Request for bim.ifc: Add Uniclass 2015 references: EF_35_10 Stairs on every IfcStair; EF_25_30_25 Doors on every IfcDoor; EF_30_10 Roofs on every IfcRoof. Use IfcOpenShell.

First a look at what the model holds.

```python
import ifcopenshell

model = ifcopenshell.open("bim.ifc")
print(model.schema)
print("classifications:", [c.Name for c in model.by_type("IfcClassification")])
for ifc_class in ("IfcDoor", "IfcRoof", "IfcStair", "IfcWall", "IfcWindow"):
    print(ifc_class, len(model.by_type(ifc_class)))
```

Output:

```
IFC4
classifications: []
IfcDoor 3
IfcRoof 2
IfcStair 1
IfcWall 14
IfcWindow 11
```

```python
import ifcopenshell
import ifcopenshell.api.classification

model = ifcopenshell.open("bim.ifc")

system = ifcopenshell.api.classification.add_classification(model, classification="Uniclass 2015")

codes = {
    "IfcStair": ("EF_35_10", "Stairs"),
    "IfcDoor": ("EF_25_30_25", "Doors"),
    "IfcRoof": ("EF_30_10", "Roofs"),
}
for ifc_class, (code, name) in codes.items():
    products = model.by_type(ifc_class)
    ifcopenshell.api.classification.add_reference(
        model, products=products, classification=system, identification=code, name=name
    )
    print(code, len(products))

model.write("bim_edited.ifc")
```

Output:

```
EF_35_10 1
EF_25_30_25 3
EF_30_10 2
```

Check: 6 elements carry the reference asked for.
